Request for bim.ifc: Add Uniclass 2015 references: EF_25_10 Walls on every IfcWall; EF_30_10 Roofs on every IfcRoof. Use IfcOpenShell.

First a look at what the model holds.

```python
import ifcopenshell

model = ifcopenshell.open("bim.ifc")
print(model.schema)
print("classifications:", [c.Name for c in model.by_type("IfcClassification")])
for ifc_class in ("IfcDoor", "IfcRoof", "IfcStair", "IfcWall", "IfcWindow"):
    print(ifc_class, len(model.by_type(ifc_class)))
```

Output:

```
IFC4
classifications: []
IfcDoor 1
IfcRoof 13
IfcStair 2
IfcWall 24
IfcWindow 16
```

```python
import ifcopenshell
import ifcopenshell.api.classification

model = ifcopenshell.open("bim.ifc")

system = ifcopenshell.api.classification.add_classification(model, classification="Uniclass 2015")

codes = {
    "IfcWall": ("EF_25_10", "Walls"),
    "IfcRoof": ("EF_30_10", "Roofs"),
}
for ifc_class, (code, name) in codes.items():
    products = model.by_type(ifc_class)
    ifcopenshell.api.classification.add_reference(
        model, products=products, classification=system, identification=code, name=name
    )
    print(code, len(products))

model.write("bim-out.ifc")
```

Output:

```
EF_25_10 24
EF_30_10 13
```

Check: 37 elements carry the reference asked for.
